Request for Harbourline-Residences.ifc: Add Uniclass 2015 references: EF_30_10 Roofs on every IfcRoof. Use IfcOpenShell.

First a look at what the model holds.

```python
import ifcopenshell

model = ifcopenshell.open("Harbourline-Residences.ifc")
print(model.schema)
print("classifications:", [c.Name for c in model.by_type("IfcClassification")])
for ifc_class in ("IfcDoor", "IfcRoof", "IfcStair", "IfcWall", "IfcWindow"):
    print(ifc_class, len(model.by_type(ifc_class)))
```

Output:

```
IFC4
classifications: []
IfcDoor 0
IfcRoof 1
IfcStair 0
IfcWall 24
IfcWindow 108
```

```python
import ifcopenshell
import ifcopenshell.api.classification

model = ifcopenshell.open("Harbourline-Residences.ifc")

system = ifcopenshell.api.classification.add_classification(model, classification="Uniclass 2015")

codes = {
    "IfcRoof": ("EF_30_10", "Roofs"),
}
for ifc_class, (code, name) in codes.items():
    products = model.by_type(ifc_class)
    ifcopenshell.api.classification.add_reference(
        model, products=products, classification=system, identification=code, name=name
    )
    print(code, len(products))

model.write("Harbourline-Residences_edited.ifc")
```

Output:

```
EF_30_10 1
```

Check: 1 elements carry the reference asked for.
